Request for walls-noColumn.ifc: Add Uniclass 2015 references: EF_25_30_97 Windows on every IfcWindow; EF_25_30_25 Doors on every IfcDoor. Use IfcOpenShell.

First a look at what the model holds.

```python
import ifcopenshell

model = ifcopenshell.open("walls-noColumn.ifc")
print(model.schema)
print("classifications:", [c.Name for c in model.by_type("IfcClassification")])
for ifc_class in ("IfcDoor", "IfcRoof", "IfcStair", "IfcWall", "IfcWindow"):
    print(ifc_class, len(model.by_type(ifc_class)))
```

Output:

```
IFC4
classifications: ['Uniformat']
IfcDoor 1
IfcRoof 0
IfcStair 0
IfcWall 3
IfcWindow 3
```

```python
import ifcopenshell
import ifcopenshell.api.classification

model = ifcopenshell.open("walls-noColumn.ifc")

system = ifcopenshell.api.classification.add_classification(model, classification="Uniclass 2015")

codes = {
    "IfcWindow": ("EF_25_30_97", "Windows"),
    "IfcDoor": ("EF_25_30_25", "Doors"),
}
for ifc_class, (code, name) in codes.items():
    products = model.by_type(ifc_class)
    ifcopenshell.api.classification.add_reference(
        model, products=products, classification=system, identification=code, name=name
    )
    print(code, len(products))

model.write("walls-noColumn_rev.ifc")
```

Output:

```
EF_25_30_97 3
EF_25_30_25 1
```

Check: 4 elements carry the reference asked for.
